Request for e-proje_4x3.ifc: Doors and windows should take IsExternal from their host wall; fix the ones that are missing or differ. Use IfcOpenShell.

First a look at what the model holds.

```python
import ifcopenshell
import ifcopenshell.util.element

model = ifcopenshell.open("e-proje_4x3.ifc")
print(model.schema)
seen = {}
for e in model.by_type("IfcDoor") + model.by_type("IfcWindow"):
    if not e.FillsVoids:
        continue
    host = e.FillsVoids[0].RelatingOpeningElement.VoidsElements[0].RelatingBuildingElement
    own = ifcopenshell.util.element.get_pset(e, f"Pset_{e.is_a()[3:].removesuffix('StandardCase')}Common", "IsExternal")
    wall = ifcopenshell.util.element.get_pset(host, "Pset_WallCommon", "IsExternal")
    seen[e.is_a(), own, wall] = seen.get((e.is_a(), own, wall), 0) + 1
for (cls, own, wall), count in sorted(seen.items(), key=str):
    print(count, cls, "IsExternal:", own, "| host wall:", wall)
```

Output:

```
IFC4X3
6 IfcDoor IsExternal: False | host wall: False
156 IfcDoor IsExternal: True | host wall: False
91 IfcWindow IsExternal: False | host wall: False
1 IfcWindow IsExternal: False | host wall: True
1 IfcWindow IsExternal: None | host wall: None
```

```python
import ifcopenshell
import ifcopenshell.api.pset
import ifcopenshell.util.element

model = ifcopenshell.open("e-proje_4x3.ifc")

count = 0
for ifc_class, pset_name in (("IfcDoor", "Pset_DoorCommon"), ("IfcWindow", "Pset_WindowCommon")):
    for e in model.by_type(ifc_class):
        if not e.FillsVoids:
            continue
        host = e.FillsVoids[0].RelatingOpeningElement.VoidsElements[0].RelatingBuildingElement
        external = ifcopenshell.util.element.get_pset(host, "Pset_WallCommon", "IsExternal")
        if external is None or ifcopenshell.util.element.get_pset(e, pset_name, "IsExternal") == external:
            continue
        pset = ifcopenshell.api.pset.add_pset(model, product=e, name=pset_name)
        ifcopenshell.api.pset.edit_pset(model, pset=pset, properties={"IsExternal": external})
        count += 1

print(count, "updated")

model.write("e-proje_4x3_updated.ifc")
```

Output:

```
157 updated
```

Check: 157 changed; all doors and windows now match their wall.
